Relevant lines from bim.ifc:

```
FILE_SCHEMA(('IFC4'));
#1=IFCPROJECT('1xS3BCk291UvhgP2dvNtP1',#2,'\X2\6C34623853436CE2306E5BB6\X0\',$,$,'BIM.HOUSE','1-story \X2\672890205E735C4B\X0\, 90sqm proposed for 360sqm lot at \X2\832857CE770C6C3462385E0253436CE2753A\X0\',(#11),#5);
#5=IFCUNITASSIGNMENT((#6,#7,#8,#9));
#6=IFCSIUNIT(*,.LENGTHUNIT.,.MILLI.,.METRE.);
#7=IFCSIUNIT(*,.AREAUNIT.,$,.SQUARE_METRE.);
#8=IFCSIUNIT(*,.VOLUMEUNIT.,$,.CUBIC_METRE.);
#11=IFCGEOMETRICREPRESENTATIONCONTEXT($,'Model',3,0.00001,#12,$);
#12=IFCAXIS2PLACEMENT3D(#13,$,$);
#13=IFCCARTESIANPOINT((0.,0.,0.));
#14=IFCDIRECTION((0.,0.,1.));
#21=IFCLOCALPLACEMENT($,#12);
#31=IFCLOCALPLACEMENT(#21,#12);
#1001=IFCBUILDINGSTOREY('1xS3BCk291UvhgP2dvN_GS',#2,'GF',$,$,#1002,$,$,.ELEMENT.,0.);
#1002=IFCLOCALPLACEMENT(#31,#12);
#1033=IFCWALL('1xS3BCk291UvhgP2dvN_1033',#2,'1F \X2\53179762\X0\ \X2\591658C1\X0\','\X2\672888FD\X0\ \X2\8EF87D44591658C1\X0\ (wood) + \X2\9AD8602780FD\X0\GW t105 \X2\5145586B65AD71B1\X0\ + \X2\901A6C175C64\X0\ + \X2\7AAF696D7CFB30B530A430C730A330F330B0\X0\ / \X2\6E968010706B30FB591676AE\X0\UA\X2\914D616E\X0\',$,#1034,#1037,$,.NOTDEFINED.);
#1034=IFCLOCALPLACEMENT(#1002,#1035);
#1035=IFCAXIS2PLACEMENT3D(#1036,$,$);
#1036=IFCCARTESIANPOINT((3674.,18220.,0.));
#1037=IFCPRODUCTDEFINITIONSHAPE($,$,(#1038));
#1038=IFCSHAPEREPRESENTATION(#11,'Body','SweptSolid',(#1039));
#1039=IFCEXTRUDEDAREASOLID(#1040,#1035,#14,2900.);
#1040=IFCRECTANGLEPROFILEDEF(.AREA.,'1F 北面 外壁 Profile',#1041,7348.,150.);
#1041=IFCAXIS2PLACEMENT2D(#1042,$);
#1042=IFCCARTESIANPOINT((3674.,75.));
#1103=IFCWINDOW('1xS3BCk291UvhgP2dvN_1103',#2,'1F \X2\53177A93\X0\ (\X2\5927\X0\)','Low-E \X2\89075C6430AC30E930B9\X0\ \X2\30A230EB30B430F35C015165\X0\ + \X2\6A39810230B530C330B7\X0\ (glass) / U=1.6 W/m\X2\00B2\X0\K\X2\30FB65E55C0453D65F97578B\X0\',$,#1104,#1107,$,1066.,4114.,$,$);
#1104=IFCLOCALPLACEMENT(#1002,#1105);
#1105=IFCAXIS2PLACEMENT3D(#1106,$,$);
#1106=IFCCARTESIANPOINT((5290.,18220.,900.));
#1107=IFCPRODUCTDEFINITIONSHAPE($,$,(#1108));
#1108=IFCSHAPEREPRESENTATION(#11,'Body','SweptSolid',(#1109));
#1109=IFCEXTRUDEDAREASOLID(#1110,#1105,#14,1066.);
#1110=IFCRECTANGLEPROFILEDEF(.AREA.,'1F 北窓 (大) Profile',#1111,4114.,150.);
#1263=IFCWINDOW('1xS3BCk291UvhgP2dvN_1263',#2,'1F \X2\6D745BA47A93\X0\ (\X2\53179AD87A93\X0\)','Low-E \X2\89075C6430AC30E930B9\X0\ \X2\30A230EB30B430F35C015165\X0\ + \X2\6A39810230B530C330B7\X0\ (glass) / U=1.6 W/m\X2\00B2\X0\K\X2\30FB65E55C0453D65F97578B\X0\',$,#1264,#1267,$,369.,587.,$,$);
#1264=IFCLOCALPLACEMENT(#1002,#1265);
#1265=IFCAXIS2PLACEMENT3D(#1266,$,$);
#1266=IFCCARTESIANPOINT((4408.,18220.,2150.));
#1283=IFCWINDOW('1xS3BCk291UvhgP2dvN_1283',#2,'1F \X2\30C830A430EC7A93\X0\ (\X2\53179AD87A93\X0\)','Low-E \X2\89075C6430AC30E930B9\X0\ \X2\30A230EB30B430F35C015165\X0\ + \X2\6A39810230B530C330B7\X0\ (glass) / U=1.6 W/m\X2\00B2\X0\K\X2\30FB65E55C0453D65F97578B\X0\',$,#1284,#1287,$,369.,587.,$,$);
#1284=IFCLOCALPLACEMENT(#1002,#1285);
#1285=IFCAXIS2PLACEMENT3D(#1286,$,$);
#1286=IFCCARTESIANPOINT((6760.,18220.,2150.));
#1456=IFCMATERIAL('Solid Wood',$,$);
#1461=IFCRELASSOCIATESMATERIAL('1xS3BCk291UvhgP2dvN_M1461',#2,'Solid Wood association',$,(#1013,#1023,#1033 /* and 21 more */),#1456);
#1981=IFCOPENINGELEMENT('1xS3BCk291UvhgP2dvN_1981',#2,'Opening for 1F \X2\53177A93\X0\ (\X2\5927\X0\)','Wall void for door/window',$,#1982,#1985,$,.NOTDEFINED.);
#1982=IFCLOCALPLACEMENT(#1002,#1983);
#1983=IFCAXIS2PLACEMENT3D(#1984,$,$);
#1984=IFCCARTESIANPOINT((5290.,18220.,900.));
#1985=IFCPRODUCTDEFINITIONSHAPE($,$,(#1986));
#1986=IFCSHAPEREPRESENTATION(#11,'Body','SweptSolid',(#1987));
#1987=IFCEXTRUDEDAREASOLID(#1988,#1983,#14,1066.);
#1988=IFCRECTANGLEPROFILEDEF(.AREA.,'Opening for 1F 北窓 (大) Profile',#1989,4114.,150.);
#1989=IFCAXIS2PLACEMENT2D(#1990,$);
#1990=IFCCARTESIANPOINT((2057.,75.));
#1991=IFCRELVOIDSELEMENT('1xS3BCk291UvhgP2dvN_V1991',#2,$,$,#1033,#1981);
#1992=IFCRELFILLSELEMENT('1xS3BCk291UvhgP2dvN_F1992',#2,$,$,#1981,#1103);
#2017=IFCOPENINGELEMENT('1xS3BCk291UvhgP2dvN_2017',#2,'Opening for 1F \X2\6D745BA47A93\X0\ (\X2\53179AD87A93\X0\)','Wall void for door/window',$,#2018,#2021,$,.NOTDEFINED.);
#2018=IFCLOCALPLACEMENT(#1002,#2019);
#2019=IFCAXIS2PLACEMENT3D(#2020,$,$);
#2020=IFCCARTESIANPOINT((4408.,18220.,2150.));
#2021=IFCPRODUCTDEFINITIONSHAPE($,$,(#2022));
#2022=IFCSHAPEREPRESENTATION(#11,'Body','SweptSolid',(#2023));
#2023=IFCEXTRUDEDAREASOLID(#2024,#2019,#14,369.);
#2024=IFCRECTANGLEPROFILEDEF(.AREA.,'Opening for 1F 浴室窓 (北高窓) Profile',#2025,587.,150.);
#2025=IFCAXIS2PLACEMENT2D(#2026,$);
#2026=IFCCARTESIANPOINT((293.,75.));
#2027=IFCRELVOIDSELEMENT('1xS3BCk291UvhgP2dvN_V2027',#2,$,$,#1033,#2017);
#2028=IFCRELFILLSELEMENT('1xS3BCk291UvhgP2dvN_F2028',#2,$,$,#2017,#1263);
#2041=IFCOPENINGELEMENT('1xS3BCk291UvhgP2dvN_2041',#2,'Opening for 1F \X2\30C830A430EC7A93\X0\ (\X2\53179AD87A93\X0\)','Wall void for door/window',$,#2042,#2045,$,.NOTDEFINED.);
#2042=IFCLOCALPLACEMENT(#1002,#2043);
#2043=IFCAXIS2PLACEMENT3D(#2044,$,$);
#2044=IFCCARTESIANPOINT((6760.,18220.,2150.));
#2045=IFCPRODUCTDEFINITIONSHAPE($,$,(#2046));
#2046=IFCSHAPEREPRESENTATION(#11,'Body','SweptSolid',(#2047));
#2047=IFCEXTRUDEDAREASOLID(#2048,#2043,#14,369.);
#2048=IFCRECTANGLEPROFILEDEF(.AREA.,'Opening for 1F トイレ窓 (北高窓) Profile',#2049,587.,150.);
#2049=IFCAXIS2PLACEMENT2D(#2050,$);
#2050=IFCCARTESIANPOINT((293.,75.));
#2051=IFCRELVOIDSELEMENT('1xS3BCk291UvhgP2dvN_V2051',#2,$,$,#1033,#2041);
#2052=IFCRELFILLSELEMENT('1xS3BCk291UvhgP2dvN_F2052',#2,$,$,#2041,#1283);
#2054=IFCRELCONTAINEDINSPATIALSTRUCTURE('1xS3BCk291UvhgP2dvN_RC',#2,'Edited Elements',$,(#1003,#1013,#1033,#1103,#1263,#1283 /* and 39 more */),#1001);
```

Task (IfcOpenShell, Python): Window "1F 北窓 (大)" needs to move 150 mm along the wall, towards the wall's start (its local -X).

```python
import ifcopenshell
import ifcopenshell.api.geometry
import ifcopenshell.util.placement
import ifcopenshell.util.unit

model = ifcopenshell.open("bim.ifc")
unit_scale = ifcopenshell.util.unit.calculate_unit_scale(model)

window = model.by_guid("1xS3BCk291UvhgP2dvN_1103")
opening = window.FillsVoids[0].RelatingOpeningElement
wall = opening.VoidsElements[0].RelatingBuildingElement

wall_matrix = ifcopenshell.util.placement.get_local_placement(wall.ObjectPlacement)
shift = wall_matrix[:3, 0] * -0.15 / unit_scale
before = ifcopenshell.util.placement.get_local_placement(window.ObjectPlacement)[:3, 3].copy()

# The window is not placed relative to its opening, so move both.
for product in (opening, window):
    matrix = ifcopenshell.util.placement.get_local_placement(product.ObjectPlacement)
    matrix[:3, 3] += shift
    ifcopenshell.api.geometry.edit_object_placement(model, product=product, matrix=matrix, is_si=False)

after = ifcopenshell.util.placement.get_local_placement(window.ObjectPlacement)[:3, 3]
print("window moved by", (after - before).round(3) + 0.0)

model.write("bim_edited.ifc")
```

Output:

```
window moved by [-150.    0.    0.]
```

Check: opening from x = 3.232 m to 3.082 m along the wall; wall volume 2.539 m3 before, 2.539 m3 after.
